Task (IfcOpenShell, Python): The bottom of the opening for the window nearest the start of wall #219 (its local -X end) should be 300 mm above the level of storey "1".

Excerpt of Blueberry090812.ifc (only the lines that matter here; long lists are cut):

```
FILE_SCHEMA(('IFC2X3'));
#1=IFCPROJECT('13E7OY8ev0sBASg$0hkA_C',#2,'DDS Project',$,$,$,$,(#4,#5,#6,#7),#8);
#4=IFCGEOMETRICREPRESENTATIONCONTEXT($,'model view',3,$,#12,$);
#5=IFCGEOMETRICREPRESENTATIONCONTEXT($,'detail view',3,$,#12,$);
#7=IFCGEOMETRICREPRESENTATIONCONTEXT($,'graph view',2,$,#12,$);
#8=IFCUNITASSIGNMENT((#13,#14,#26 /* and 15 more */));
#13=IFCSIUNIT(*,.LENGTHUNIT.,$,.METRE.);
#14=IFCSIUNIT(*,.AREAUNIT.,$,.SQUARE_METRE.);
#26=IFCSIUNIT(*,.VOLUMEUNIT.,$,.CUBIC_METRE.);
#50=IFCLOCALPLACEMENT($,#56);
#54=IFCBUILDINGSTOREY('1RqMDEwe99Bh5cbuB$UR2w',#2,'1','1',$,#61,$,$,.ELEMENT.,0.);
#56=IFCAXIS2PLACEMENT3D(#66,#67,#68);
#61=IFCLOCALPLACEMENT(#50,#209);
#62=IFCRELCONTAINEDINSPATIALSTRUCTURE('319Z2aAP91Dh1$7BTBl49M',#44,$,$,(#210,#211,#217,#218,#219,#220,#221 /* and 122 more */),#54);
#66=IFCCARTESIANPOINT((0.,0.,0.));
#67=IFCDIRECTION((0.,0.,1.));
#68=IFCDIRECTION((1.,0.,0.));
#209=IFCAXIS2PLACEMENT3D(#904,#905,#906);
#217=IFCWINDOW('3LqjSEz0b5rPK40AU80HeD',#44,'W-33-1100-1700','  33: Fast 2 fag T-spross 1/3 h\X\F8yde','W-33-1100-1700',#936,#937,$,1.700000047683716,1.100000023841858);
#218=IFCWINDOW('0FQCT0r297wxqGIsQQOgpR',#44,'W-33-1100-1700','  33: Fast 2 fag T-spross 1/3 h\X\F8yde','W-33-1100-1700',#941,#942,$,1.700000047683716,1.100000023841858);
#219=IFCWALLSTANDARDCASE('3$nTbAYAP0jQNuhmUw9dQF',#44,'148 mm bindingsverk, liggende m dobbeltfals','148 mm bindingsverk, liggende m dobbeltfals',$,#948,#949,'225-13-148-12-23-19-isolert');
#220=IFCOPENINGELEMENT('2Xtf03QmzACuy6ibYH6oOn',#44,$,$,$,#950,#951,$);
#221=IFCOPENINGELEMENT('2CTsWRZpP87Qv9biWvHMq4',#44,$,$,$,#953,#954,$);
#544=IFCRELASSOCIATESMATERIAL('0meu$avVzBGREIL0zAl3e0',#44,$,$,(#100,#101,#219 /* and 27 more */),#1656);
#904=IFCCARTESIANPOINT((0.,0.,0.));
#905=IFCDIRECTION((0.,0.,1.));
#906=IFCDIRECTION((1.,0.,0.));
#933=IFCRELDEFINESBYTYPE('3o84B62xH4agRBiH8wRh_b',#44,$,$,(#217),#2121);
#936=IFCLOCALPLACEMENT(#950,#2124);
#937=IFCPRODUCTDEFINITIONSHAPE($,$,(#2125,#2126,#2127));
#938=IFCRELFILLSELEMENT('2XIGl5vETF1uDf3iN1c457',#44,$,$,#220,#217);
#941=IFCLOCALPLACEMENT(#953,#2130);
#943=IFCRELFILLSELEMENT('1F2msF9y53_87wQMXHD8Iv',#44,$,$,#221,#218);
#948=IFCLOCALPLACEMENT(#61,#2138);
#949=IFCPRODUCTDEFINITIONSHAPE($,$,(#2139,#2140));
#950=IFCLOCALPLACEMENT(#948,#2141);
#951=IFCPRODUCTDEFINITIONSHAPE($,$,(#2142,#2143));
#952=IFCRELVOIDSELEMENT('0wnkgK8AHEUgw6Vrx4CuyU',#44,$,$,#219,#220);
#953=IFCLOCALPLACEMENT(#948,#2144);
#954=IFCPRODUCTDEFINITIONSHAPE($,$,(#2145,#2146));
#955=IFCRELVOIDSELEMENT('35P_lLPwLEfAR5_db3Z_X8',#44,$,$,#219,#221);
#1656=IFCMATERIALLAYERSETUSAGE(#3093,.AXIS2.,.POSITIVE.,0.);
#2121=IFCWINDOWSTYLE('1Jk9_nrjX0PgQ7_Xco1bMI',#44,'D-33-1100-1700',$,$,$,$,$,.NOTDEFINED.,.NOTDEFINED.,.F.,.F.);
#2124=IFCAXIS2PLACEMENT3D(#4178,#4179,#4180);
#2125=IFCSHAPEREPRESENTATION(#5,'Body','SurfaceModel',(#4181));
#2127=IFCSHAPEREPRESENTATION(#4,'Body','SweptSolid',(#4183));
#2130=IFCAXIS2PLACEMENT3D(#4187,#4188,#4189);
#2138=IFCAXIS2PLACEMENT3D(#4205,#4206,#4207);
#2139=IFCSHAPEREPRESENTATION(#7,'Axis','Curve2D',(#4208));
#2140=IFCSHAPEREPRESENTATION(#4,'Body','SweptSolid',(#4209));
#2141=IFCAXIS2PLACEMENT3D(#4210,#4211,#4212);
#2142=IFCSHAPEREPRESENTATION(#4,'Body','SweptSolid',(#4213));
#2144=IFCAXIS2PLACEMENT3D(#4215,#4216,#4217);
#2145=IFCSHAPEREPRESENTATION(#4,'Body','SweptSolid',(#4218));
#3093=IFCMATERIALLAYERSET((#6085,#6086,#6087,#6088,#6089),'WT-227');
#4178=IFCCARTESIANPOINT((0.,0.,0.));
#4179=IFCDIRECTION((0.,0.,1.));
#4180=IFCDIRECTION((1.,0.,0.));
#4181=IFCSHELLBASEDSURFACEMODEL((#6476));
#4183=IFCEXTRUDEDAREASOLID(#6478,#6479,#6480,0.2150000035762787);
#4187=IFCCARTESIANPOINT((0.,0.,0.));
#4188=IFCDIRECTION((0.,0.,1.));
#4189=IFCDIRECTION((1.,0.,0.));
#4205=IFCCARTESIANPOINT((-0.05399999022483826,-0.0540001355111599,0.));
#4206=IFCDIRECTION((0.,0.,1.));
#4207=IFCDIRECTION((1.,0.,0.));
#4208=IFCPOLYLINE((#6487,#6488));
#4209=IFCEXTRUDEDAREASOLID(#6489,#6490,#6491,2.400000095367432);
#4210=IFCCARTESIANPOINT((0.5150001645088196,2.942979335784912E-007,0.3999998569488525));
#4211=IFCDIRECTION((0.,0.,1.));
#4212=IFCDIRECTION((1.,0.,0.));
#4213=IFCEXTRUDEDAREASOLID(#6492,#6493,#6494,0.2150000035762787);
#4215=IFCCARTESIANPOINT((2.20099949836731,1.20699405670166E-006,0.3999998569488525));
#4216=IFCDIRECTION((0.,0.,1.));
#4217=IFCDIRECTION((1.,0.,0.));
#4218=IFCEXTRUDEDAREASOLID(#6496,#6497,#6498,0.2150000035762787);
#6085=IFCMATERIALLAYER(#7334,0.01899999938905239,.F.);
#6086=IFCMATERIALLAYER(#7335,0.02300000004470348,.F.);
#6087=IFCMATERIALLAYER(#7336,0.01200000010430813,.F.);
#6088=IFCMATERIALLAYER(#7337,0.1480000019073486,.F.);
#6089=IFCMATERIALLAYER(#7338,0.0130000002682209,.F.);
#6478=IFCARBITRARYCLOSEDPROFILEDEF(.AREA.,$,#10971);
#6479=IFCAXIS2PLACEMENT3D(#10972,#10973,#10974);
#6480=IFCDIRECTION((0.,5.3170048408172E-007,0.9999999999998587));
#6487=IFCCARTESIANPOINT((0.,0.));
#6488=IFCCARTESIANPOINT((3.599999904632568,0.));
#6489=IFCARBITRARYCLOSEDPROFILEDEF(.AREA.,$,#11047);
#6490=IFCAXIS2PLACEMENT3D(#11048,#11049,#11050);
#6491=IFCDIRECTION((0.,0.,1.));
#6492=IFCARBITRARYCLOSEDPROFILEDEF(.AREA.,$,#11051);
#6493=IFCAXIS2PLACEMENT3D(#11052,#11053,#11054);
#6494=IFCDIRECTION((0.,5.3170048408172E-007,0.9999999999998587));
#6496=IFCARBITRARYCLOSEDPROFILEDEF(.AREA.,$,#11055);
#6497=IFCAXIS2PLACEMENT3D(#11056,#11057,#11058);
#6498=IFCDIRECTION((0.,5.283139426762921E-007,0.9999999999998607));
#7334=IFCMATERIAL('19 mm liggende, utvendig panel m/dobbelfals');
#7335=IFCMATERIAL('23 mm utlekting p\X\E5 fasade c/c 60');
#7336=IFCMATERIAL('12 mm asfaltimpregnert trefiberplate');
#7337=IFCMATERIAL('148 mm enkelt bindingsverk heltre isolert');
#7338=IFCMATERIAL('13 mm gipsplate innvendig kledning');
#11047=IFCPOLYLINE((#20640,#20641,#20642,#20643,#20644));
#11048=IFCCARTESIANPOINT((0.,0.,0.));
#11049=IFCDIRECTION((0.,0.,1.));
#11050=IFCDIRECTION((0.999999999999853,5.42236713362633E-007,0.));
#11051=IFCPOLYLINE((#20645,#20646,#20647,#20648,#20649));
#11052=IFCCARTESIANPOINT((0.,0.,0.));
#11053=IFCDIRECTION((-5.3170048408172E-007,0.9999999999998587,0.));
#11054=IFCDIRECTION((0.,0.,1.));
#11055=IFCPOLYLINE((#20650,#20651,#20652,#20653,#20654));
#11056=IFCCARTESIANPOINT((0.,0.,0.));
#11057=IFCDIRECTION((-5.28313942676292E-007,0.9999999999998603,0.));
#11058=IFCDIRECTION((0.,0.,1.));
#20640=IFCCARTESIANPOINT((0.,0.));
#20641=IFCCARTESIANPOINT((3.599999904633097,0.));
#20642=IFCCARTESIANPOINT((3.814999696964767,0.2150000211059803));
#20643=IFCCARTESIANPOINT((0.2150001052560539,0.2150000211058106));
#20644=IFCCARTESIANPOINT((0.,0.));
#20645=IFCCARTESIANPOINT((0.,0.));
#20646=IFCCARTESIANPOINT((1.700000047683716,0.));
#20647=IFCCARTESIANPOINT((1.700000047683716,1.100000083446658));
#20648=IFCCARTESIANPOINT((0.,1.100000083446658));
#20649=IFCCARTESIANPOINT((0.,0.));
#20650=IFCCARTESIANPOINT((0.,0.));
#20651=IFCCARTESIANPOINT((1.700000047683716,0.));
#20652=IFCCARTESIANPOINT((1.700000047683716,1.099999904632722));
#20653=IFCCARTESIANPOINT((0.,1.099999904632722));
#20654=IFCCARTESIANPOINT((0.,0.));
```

```python
import numpy as np
import ifcopenshell
import ifcopenshell.api.geometry
import ifcopenshell.geom
import ifcopenshell.util.element
import ifcopenshell.util.placement
import ifcopenshell.util.shape
import ifcopenshell.util.unit

model = ifcopenshell.open("Blueberry090812.ifc")
unit_scale = ifcopenshell.util.unit.calculate_unit_scale(model)

window = model.by_guid("3LqjSEz0b5rPK40AU80HeD")
opening = window.FillsVoids[0].RelatingOpeningElement
storey = ifcopenshell.util.element.get_container(window, ifc_class="IfcBuildingStorey")
level = ifcopenshell.util.placement.get_local_placement(storey.ObjectPlacement)[2, 3]

# The opening's origin need not be at the sill, so measure its lowest point.
shape = ifcopenshell.geom.create_shape(ifcopenshell.geom.settings(), opening)
bottom = ifcopenshell.util.shape.get_shape_bottom_elevation(shape, shape.geometry) / unit_scale
dz = level + 0.3 / unit_scale - bottom

shift = np.array([0.0, 0.0, dz])
# The window is placed relative to its opening, so it follows when the opening moves.
matrix = ifcopenshell.util.placement.get_local_placement(opening.ObjectPlacement)
matrix[:3, 3] += shift
ifcopenshell.api.geometry.edit_object_placement(
    model, product=opening, matrix=matrix, is_si=False, should_transform_children=True
)

print(f"moved by {dz * unit_scale:+.3f} m")

model.write("Blueberry090812_edited.ifc")
```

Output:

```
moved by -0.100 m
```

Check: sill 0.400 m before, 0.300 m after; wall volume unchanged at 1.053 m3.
